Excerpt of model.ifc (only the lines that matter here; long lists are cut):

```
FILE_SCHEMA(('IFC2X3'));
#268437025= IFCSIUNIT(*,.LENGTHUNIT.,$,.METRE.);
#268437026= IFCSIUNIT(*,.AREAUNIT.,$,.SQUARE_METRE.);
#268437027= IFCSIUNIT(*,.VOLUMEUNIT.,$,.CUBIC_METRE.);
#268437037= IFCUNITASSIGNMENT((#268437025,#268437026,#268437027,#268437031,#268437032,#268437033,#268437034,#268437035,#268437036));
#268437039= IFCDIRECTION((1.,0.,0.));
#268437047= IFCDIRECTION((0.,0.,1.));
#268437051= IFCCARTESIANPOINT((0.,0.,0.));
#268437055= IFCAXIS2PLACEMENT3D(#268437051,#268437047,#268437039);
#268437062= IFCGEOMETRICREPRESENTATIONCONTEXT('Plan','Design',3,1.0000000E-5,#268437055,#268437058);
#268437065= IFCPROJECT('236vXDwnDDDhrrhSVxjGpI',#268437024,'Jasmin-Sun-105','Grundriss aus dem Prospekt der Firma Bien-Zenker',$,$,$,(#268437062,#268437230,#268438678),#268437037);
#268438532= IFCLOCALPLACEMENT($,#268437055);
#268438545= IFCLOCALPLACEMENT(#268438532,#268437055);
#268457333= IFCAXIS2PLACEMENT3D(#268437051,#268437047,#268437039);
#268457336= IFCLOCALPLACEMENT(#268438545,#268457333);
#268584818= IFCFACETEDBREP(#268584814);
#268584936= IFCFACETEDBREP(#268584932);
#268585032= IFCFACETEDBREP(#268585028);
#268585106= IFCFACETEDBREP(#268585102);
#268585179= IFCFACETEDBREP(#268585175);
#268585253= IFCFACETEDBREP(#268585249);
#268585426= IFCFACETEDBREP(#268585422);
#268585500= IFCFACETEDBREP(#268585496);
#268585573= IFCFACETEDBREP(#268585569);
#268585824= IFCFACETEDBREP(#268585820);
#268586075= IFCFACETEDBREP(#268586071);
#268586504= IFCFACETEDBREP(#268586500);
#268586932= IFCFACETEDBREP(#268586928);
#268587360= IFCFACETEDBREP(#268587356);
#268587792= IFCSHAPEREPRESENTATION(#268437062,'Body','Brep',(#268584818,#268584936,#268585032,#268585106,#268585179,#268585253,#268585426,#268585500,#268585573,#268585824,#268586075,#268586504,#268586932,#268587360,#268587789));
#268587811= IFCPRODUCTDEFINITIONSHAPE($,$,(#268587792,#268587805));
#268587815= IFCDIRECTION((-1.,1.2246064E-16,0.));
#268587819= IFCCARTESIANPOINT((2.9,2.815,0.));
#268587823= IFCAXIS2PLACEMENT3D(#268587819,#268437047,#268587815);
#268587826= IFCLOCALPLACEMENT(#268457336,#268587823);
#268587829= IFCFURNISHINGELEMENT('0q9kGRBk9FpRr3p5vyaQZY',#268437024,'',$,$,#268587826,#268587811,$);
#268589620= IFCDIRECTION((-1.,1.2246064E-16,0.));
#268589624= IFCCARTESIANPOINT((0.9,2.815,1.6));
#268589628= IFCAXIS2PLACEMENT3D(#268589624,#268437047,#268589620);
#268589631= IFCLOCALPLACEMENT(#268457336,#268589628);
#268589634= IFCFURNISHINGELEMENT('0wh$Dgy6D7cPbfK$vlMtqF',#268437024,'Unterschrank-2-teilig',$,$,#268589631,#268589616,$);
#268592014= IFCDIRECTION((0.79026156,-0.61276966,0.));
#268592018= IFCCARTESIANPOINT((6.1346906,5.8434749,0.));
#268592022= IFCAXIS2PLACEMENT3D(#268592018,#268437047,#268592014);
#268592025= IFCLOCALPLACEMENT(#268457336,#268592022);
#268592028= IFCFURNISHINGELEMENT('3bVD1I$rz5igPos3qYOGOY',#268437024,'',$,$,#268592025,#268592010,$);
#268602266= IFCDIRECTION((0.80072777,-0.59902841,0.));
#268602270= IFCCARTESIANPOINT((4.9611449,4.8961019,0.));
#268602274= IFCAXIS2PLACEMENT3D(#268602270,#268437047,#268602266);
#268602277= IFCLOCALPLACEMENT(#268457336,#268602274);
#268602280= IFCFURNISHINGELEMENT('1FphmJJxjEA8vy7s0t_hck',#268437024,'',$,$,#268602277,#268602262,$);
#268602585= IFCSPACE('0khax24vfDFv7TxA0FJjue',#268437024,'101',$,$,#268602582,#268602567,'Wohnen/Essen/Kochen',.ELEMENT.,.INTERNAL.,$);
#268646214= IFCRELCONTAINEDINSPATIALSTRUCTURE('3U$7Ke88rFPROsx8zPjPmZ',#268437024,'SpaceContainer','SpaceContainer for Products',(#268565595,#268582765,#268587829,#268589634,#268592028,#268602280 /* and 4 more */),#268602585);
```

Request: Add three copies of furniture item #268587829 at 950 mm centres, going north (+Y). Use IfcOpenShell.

```python
import numpy as np
import ifcopenshell
import ifcopenshell.api.geometry
import ifcopenshell.api.root
import ifcopenshell.util.element
import ifcopenshell.util.placement
import ifcopenshell.util.unit

model = ifcopenshell.open("model.ifc")
unit_scale = ifcopenshell.util.unit.calculate_unit_scale(model)


def reuse_history(source, copy):
    """copy_class also copies each property set's owner history, people and application; keep the originals."""
    for rel in copy.IsDefinedBy:
        if rel.is_a("IfcRelDefinesByProperties") and (history := rel.RelatingPropertyDefinition.OwnerHistory):
            rel.RelatingPropertyDefinition.OwnerHistory = source.OwnerHistory
            ifcopenshell.util.element.remove_deep2(model, history)


source = model.by_guid("0q9kGRBk9FpRr3p5vyaQZY")
base = ifcopenshell.util.placement.get_local_placement(source.ObjectPlacement)
step = np.array([0.0, 1.0, 0.0]) * 0.95 / unit_scale

for i in range(1, 4):
    copy = ifcopenshell.api.root.copy_class(model, product=source)
    copy.Representation = ifcopenshell.util.element.copy_deep(
        model, source.Representation, exclude=["IfcGeometricRepresentationContext", "IfcRepresentationMap"]
    )
    reuse_history(source, copy)
    matrix = base.copy()
    matrix[:3, 3] += i * step
    print("added at", matrix[:3, 3].round(3) + 0.0)
    ifcopenshell.api.geometry.edit_object_placement(model, product=copy, matrix=matrix, is_si=False)

model.write("model_updated.ifc")
```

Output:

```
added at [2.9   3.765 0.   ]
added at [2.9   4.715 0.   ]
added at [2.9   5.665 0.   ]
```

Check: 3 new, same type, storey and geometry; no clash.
